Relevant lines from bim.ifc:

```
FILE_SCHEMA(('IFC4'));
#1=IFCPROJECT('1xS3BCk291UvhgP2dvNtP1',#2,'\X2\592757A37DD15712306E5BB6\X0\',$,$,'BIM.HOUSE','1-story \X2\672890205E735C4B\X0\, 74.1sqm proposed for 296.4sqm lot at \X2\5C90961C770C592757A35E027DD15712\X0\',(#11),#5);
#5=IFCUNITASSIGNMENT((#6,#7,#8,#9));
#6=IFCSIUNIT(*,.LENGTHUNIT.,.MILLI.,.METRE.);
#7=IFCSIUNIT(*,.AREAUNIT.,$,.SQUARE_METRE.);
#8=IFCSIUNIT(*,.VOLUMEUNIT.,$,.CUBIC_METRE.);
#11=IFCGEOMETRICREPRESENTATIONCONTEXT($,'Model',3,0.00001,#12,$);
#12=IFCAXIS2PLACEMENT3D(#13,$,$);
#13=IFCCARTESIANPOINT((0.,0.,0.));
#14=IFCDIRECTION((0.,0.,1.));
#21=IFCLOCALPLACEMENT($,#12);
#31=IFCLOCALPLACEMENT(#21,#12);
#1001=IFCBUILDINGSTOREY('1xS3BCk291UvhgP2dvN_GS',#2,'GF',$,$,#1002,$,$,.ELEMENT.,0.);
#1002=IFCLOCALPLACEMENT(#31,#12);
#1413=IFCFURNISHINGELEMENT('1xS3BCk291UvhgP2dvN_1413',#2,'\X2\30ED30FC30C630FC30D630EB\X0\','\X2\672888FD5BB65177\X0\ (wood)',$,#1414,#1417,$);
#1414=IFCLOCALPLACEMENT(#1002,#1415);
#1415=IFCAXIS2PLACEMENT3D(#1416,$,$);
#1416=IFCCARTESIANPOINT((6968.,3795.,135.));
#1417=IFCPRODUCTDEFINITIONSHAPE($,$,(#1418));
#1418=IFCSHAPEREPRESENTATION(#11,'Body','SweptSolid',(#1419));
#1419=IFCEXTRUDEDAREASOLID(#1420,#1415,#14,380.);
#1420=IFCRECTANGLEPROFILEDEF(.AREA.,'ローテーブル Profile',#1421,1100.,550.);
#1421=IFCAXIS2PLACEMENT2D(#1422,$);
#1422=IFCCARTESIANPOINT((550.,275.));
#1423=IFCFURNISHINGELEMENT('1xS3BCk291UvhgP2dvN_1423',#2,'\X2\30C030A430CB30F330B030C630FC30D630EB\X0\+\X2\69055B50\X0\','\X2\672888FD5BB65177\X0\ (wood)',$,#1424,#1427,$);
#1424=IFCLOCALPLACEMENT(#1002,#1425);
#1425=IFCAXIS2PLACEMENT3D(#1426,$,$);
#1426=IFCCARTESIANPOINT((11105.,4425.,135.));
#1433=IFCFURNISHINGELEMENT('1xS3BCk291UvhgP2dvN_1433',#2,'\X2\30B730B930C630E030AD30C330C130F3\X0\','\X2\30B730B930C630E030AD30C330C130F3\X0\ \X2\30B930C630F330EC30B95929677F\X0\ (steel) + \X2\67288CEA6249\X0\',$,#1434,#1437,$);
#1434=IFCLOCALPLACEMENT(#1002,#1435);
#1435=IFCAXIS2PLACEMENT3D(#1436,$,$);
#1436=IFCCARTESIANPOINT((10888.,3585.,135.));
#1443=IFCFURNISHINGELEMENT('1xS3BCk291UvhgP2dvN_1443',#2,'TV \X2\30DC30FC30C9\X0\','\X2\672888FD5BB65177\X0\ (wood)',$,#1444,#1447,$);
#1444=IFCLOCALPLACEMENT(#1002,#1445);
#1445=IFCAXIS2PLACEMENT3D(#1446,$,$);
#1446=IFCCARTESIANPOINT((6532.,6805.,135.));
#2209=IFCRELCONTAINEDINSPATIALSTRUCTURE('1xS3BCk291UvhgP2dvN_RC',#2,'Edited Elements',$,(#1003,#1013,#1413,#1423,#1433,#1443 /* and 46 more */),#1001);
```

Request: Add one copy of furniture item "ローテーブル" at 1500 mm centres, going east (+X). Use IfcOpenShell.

```python
import numpy as np
import ifcopenshell
import ifcopenshell.api.geometry
import ifcopenshell.api.root
import ifcopenshell.util.element
import ifcopenshell.util.placement
import ifcopenshell.util.unit

model = ifcopenshell.open("bim.ifc")
unit_scale = ifcopenshell.util.unit.calculate_unit_scale(model)


def reuse_history(source, copy):
    """copy_class also copies each property set's owner history, people and application; keep the originals."""
    for rel in copy.IsDefinedBy:
        if rel.is_a("IfcRelDefinesByProperties") and (history := rel.RelatingPropertyDefinition.OwnerHistory):
            rel.RelatingPropertyDefinition.OwnerHistory = source.OwnerHistory
            ifcopenshell.util.element.remove_deep2(model, history)


source = model.by_id(1413)
base = ifcopenshell.util.placement.get_local_placement(source.ObjectPlacement)
step = np.array([1.0, 0.0, 0.0]) * 1.5 / unit_scale

for i in range(1, 2):
    copy = ifcopenshell.api.root.copy_class(model, product=source)
    copy.Representation = ifcopenshell.util.element.copy_deep(
        model, source.Representation, exclude=["IfcGeometricRepresentationContext", "IfcRepresentationMap"]
    )
    reuse_history(source, copy)
    matrix = base.copy()
    matrix[:3, 3] += i * step
    print("added at", matrix[:3, 3].round(3) + 0.0)
    ifcopenshell.api.geometry.edit_object_placement(model, product=copy, matrix=matrix, is_si=False)

model.write("bim_rev.ifc")
```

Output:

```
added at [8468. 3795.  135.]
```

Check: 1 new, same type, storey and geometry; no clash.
